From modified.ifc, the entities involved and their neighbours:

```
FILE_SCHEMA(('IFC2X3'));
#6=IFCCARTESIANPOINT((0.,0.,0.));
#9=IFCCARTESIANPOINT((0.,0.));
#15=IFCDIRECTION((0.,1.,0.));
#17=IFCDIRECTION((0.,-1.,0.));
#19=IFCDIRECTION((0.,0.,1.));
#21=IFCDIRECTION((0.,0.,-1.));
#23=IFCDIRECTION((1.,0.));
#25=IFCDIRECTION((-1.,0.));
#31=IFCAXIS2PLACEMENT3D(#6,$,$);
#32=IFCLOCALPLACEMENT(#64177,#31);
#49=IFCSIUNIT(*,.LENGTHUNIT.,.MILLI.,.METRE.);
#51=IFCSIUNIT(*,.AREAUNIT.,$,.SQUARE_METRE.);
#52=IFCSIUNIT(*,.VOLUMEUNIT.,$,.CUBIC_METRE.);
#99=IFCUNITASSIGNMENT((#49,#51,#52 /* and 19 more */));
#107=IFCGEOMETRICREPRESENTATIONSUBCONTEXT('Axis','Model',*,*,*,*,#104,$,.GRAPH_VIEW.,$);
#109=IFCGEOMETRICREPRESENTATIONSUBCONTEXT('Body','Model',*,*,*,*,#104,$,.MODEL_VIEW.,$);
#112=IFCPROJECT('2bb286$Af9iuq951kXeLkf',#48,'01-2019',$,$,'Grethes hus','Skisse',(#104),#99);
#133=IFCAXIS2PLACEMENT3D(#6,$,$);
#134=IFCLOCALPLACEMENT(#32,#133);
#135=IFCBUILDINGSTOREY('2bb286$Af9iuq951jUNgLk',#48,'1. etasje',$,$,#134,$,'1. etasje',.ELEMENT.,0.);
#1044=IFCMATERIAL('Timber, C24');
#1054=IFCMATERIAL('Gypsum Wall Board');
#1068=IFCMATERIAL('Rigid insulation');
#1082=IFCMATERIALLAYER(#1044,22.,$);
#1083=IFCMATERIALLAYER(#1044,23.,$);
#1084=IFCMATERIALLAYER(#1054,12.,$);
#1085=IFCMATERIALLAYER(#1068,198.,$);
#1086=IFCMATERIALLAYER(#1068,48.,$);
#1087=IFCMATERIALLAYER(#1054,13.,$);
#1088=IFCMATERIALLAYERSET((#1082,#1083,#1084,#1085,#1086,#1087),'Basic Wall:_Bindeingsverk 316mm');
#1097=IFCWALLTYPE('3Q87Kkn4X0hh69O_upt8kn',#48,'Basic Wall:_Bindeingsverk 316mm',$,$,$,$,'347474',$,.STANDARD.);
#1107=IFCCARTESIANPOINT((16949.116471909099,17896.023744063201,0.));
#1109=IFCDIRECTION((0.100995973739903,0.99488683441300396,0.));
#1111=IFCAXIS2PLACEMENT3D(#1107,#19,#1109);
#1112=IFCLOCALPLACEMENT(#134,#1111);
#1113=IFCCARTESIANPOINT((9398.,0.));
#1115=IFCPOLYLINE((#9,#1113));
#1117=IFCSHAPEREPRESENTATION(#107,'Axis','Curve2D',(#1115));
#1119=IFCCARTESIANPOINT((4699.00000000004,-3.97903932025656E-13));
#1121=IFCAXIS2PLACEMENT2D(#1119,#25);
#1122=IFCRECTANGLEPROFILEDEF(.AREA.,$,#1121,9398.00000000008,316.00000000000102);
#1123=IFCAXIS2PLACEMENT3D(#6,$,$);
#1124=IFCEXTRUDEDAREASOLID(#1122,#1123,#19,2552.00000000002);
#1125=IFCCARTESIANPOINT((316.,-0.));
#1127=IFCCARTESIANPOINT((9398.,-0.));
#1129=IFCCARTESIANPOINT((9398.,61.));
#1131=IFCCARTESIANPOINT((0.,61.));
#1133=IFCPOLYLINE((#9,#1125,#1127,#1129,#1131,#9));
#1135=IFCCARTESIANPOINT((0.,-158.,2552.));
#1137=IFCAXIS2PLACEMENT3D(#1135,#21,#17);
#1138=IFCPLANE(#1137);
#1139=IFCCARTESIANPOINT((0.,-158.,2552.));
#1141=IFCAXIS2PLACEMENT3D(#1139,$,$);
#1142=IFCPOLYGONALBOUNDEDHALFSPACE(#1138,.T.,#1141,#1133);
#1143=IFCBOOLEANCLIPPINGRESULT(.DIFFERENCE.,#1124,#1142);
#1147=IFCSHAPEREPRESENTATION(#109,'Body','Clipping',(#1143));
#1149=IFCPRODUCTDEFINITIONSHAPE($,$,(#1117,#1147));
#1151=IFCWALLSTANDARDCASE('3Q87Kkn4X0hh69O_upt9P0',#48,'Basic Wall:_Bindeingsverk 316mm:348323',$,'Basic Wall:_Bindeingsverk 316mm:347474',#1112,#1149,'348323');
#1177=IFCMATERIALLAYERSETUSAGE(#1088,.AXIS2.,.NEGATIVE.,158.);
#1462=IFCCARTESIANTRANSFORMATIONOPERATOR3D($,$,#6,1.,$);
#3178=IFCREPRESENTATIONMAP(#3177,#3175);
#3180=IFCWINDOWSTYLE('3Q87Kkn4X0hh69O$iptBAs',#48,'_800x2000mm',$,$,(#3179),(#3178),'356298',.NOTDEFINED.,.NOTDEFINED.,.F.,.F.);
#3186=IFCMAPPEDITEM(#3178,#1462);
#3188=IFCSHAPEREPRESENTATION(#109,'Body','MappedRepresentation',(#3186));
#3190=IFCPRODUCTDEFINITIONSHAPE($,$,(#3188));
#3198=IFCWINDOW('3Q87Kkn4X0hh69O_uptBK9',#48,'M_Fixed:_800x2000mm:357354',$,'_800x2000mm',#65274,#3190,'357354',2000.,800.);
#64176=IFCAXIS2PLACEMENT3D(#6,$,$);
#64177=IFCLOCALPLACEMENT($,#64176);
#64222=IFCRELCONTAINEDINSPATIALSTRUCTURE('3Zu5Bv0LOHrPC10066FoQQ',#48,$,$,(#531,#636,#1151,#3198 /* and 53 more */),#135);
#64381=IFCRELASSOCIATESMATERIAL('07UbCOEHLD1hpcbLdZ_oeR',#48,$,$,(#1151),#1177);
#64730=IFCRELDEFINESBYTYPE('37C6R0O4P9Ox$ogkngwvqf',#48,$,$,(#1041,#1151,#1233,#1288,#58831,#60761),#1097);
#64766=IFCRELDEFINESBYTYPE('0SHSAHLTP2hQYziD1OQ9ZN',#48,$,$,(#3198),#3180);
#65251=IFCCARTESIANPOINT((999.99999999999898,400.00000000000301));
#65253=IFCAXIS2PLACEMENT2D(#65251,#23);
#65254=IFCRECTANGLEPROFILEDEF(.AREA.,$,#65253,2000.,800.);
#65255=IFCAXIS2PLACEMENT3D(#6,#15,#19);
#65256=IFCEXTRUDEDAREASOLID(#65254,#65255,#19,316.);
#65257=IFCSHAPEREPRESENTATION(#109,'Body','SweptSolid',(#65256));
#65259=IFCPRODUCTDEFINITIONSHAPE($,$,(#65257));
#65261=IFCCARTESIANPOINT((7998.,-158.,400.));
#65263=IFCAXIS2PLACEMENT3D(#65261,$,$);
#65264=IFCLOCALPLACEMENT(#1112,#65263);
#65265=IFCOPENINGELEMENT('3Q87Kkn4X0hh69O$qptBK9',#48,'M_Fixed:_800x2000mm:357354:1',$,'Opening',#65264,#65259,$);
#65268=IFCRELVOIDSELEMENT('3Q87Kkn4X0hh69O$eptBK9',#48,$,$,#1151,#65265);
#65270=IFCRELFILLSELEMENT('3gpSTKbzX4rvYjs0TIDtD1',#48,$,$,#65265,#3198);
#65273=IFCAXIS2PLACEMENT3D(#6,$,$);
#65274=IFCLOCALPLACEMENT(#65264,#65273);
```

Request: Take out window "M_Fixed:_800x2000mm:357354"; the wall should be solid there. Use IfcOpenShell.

```python
import ifcopenshell
import ifcopenshell.api.feature
import ifcopenshell.api.root
import ifcopenshell.geom
import ifcopenshell.util.shape

model = ifcopenshell.open("modified.ifc")
settings = ifcopenshell.geom.settings()


def volume(element):
    """Net volume in cubic metres, openings subtracted."""
    shape = ifcopenshell.geom.create_shape(settings, element)
    return ifcopenshell.util.shape.get_volume(shape.geometry)


window = model.by_guid("3Q87Kkn4X0hh69O_uptBK9")
opening = window.FillsVoids[0].RelatingOpeningElement
wall = opening.VoidsElements[0].RelatingBuildingElement
before = volume(wall)

ifcopenshell.api.root.remove_product(model, product=window)
ifcopenshell.api.feature.remove_feature(model, feature=opening)

after = volume(wall)

print(f"wall volume {before:.3f} -> {after:.3f} m3")

model.write("modified_v2.ifc")
```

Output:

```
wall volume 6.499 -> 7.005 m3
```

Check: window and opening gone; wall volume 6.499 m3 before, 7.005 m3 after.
